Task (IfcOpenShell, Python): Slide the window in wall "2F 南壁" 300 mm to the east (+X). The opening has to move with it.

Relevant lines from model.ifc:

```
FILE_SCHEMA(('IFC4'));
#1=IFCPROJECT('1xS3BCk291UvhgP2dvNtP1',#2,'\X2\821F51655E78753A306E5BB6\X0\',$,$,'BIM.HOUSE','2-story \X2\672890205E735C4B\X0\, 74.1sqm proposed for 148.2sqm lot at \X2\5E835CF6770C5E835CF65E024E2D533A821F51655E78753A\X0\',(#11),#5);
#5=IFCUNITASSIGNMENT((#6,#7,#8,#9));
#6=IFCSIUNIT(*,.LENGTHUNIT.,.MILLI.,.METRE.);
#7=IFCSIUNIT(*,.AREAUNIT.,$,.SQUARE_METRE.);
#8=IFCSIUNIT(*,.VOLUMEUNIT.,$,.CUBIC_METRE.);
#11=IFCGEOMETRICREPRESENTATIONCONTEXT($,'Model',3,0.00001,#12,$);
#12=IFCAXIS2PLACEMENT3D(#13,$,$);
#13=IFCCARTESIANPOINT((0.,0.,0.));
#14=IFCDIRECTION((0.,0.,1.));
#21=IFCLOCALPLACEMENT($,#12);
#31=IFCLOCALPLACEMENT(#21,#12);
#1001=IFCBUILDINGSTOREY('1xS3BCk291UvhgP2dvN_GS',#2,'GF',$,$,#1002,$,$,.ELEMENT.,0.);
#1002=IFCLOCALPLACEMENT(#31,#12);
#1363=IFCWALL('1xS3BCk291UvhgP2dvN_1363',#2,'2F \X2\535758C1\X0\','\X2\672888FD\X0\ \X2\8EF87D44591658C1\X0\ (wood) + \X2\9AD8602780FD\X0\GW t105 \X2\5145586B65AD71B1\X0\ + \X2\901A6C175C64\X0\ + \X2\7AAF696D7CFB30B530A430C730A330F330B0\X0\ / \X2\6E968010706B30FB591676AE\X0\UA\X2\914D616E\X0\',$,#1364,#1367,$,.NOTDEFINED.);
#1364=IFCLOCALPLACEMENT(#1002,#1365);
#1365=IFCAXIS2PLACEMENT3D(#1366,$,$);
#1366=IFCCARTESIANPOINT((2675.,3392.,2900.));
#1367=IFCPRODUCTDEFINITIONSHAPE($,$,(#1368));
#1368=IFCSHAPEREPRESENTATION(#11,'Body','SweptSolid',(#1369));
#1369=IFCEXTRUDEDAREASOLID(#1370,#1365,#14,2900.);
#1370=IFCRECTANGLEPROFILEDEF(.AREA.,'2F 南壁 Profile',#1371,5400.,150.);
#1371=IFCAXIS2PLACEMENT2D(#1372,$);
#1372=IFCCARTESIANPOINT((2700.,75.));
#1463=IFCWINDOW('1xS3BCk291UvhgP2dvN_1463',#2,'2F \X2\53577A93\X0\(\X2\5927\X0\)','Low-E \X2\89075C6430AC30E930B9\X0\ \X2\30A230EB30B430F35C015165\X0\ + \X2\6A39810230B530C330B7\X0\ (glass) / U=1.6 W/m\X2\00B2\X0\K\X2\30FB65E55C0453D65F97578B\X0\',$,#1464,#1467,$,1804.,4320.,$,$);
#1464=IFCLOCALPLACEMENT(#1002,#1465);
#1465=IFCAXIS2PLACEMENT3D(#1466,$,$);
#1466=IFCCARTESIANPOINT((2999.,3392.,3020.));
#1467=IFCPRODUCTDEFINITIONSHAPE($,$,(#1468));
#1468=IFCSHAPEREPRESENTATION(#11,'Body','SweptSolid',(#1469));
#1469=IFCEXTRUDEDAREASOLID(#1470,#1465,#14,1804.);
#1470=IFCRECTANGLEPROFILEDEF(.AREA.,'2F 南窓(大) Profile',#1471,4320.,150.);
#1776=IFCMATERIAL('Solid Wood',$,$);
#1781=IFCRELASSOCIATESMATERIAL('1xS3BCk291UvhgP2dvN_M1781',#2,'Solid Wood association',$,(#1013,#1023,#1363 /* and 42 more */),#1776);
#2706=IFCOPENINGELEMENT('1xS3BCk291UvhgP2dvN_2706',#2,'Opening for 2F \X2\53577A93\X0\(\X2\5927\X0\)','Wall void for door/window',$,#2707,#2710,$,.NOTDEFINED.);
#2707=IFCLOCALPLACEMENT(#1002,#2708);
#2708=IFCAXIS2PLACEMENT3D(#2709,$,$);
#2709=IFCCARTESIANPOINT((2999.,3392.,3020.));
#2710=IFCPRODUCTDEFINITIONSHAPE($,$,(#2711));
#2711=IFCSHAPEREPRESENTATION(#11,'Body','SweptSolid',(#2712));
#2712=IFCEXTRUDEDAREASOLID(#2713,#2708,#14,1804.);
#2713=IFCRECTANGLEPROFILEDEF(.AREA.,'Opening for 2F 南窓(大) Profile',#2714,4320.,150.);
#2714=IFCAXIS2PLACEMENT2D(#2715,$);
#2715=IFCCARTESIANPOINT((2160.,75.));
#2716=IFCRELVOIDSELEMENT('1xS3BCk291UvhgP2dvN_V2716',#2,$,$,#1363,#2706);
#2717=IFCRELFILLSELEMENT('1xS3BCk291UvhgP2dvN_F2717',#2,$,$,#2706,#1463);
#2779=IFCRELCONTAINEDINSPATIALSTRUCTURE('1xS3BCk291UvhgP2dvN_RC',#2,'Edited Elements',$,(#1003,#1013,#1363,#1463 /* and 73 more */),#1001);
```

```python
import ifcopenshell
import ifcopenshell.api.geometry
import ifcopenshell.util.placement
import ifcopenshell.util.unit

model = ifcopenshell.open("model.ifc")
unit_scale = ifcopenshell.util.unit.calculate_unit_scale(model)

window = model.by_guid("1xS3BCk291UvhgP2dvN_1463")
opening = window.FillsVoids[0].RelatingOpeningElement
wall = opening.VoidsElements[0].RelatingBuildingElement

wall_matrix = ifcopenshell.util.placement.get_local_placement(wall.ObjectPlacement)
shift = wall_matrix[:3, 0] * 0.3 / unit_scale
before = ifcopenshell.util.placement.get_local_placement(window.ObjectPlacement)[:3, 3].copy()

# The window is not placed relative to its opening, so move both.
for product in (opening, window):
    matrix = ifcopenshell.util.placement.get_local_placement(product.ObjectPlacement)
    matrix[:3, 3] += shift
    ifcopenshell.api.geometry.edit_object_placement(model, product=product, matrix=matrix, is_si=False)

after = ifcopenshell.util.placement.get_local_placement(window.ObjectPlacement)[:3, 3]
print("window moved by", (after - before).round(3) + 0.0)

model.write("model_v2.ifc")
```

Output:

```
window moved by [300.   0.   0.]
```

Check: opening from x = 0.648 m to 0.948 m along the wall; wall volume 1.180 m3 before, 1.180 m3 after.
